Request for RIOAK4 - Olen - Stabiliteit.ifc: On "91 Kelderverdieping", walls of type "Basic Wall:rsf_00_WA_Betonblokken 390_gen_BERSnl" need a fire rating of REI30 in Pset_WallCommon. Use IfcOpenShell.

First a look at what the model holds.

```python
import ifcopenshell
import ifcopenshell.util.element

model = ifcopenshell.open("RIOAK4 - Olen - Stabiliteit.ifc")
print(model.schema)
storey = next(s for s in model.by_type("IfcBuildingStorey") if s.Name == "91 Kelderverdieping")
walls = [e for e in ifcopenshell.util.element.get_decomposition(storey) if e.is_a("IfcWall")]
seen = {}
for e in walls:
    element_type = ifcopenshell.util.element.get_type(e)
    key = (element_type.Name if element_type != e and element_type else None, ifcopenshell.util.element.get_pset(e, "Pset_WallCommon", "FireRating"))
    seen[key] = seen.get(key, 0) + 1
for (name, value), count in sorted(seen.items(), key=str):
    print(count, "x", name, "|", value)
```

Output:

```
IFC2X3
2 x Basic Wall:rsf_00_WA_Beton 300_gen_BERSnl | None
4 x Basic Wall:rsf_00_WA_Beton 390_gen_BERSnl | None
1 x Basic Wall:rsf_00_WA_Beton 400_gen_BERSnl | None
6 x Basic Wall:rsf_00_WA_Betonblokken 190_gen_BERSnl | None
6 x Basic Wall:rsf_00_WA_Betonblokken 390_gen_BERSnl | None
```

```python
import ifcopenshell
import ifcopenshell.api.pset
import ifcopenshell.util.element

model = ifcopenshell.open("RIOAK4 - Olen - Stabiliteit.ifc")

storey = next(s for s in model.by_type("IfcBuildingStorey") if s.Name == "91 Kelderverdieping")
walls = [e for e in ifcopenshell.util.element.get_decomposition(storey) if e.is_a("IfcWall")]

count = 0
for e in walls:
    element_type = ifcopenshell.util.element.get_type(e)
    if element_type in (None, e) or element_type.Name != "Basic Wall:rsf_00_WA_Betonblokken 390_gen_BERSnl":
        continue
    # add_pset returns the element's existing set when there is one.
    pset = ifcopenshell.api.pset.add_pset(model, product=e, name="Pset_WallCommon")
    ifcopenshell.api.pset.edit_pset(model, pset=pset, properties={"FireRating": "REI30"})
    count += 1

print(count, "walls updated")

model.write("RIOAK4 - Olen - Stabiliteit_rev.ifc")
```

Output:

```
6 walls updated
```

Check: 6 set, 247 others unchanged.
